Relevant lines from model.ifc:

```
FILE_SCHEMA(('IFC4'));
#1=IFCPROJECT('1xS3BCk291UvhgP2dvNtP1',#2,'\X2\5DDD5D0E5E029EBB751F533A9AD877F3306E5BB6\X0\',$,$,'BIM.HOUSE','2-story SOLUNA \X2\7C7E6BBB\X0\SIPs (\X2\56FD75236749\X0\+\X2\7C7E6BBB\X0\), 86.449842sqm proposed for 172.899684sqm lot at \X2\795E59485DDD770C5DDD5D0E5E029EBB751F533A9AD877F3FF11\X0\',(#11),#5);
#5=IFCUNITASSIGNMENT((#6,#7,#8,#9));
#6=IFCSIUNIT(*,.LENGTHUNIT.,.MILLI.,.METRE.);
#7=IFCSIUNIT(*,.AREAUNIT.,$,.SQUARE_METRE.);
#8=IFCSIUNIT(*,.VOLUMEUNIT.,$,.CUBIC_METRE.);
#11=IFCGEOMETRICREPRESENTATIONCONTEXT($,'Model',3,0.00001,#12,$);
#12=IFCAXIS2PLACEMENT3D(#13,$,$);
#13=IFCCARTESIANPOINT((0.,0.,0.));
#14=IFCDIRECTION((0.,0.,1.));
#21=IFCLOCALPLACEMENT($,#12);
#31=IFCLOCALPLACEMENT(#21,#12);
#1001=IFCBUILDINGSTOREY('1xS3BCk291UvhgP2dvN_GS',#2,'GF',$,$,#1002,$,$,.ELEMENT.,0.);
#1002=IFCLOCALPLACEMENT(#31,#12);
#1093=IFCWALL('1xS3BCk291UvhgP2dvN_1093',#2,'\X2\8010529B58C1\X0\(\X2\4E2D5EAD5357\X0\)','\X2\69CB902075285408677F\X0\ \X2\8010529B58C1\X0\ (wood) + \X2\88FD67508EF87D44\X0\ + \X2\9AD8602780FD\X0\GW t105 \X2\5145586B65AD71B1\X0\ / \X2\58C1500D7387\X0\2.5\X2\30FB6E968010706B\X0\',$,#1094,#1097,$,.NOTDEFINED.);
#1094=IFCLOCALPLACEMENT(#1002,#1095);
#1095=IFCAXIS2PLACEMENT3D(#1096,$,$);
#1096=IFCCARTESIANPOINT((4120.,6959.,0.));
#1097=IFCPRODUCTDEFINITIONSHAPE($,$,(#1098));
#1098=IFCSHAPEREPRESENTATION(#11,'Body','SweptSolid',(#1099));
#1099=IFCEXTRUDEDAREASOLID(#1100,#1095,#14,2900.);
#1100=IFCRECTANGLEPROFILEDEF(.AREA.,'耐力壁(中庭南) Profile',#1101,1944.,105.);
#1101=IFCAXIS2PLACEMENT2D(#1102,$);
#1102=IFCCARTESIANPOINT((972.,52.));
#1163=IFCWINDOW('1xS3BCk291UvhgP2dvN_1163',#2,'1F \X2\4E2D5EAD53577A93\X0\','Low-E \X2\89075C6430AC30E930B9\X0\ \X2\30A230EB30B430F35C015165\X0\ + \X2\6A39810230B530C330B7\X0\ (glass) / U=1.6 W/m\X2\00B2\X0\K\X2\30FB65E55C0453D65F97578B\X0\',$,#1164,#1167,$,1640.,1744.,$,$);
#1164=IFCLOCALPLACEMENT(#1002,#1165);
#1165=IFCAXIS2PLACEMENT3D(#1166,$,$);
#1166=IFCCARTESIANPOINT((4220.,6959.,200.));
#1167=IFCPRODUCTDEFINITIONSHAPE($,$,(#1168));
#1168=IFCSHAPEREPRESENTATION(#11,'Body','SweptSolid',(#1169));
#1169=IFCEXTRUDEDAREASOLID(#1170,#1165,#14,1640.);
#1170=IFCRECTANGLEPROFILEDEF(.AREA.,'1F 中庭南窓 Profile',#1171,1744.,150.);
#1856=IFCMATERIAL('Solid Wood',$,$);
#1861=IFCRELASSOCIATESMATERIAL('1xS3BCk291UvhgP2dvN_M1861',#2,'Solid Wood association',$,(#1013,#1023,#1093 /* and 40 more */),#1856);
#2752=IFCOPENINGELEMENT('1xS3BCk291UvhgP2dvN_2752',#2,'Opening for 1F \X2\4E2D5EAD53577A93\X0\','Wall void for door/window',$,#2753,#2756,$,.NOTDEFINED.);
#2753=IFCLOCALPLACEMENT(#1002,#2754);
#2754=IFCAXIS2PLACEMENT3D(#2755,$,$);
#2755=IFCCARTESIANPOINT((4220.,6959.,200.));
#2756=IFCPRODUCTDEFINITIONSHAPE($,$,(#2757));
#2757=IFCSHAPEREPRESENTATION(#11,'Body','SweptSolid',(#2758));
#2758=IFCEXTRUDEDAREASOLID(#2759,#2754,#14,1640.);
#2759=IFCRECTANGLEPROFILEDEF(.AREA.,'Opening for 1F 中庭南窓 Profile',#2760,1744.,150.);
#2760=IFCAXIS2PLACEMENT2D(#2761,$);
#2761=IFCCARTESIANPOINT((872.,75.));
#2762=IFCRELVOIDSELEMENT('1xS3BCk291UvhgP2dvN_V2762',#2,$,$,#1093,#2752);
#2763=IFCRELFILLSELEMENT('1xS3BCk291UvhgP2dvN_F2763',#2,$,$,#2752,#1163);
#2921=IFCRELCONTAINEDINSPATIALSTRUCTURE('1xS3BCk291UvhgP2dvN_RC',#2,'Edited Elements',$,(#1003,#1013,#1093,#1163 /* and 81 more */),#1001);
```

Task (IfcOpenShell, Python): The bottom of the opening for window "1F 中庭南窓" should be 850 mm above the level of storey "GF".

```python
import numpy as np
import ifcopenshell
import ifcopenshell.api.geometry
import ifcopenshell.geom
import ifcopenshell.util.element
import ifcopenshell.util.placement
import ifcopenshell.util.shape
import ifcopenshell.util.unit

model = ifcopenshell.open("model.ifc")
unit_scale = ifcopenshell.util.unit.calculate_unit_scale(model)

window = model.by_guid("1xS3BCk291UvhgP2dvN_1163")
opening = window.FillsVoids[0].RelatingOpeningElement
storey = ifcopenshell.util.element.get_container(window, ifc_class="IfcBuildingStorey")
level = ifcopenshell.util.placement.get_local_placement(storey.ObjectPlacement)[2, 3]

# The opening's origin need not be at the sill, so measure its lowest point.
shape = ifcopenshell.geom.create_shape(ifcopenshell.geom.settings(), opening)
bottom = ifcopenshell.util.shape.get_shape_bottom_elevation(shape, shape.geometry) / unit_scale
dz = level + 850.0 - bottom

shift = np.array([0.0, 0.0, dz])
# The window is not placed relative to its opening, so move both.
for product in (opening, window):
    matrix = ifcopenshell.util.placement.get_local_placement(product.ObjectPlacement)
    matrix[:3, 3] += shift
    ifcopenshell.api.geometry.edit_object_placement(model, product=product, matrix=matrix, is_si=False)

print(f"moved by {dz * unit_scale:+.3f} m")

model.write("model_edited.ifc")
```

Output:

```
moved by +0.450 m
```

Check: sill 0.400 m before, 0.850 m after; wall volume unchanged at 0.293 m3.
